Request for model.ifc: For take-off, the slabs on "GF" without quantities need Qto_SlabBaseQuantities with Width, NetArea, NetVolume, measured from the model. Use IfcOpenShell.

First a look at what the model holds.

```python
import ifcopenshell
import ifcopenshell.util.element
import ifcopenshell.util.unit

model = ifcopenshell.open("model.ifc")
print(model.schema)
for unit_type in ("LENGTHUNIT", "AREAUNIT", "VOLUMEUNIT"):
    print(unit_type, ifcopenshell.util.unit.calculate_unit_scale(model, unit_type))
storey = next(s for s in model.by_type("IfcBuildingStorey") if s.Name == "GF")
slabs = [e for e in ifcopenshell.util.element.get_decomposition(storey) if e.is_a("IfcSlab")]
for e in sorted(slabs, key=lambda e: e.id()):
    print(e.id(), e.is_a(), e.Name, list(ifcopenshell.util.element.get_psets(e, qtos_only=True)), sep=" | ")
```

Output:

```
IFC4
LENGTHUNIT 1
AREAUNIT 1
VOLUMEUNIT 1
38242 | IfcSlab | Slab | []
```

```python
import ifcopenshell
import ifcopenshell.api.pset
import ifcopenshell.geom
import ifcopenshell.util.element
import ifcopenshell.util.shape
import ifcopenshell.util.unit

model = ifcopenshell.open("model.ifc")
unit_scale = ifcopenshell.util.unit.calculate_unit_scale(model)
area_scale = ifcopenshell.util.unit.calculate_unit_scale(model, "AREAUNIT")
volume_scale = ifcopenshell.util.unit.calculate_unit_scale(model, "VOLUMEUNIT")
settings = ifcopenshell.geom.settings()

storey = next(s for s in model.by_type("IfcBuildingStorey") if s.Name == "GF")
slabs = [e for e in ifcopenshell.util.element.get_decomposition(storey) if e.is_a("IfcSlab")]

for e in sorted(slabs, key=lambda e: e.id()):
    if ifcopenshell.util.element.get_psets(e, qtos_only=True, should_inherit=False):
        continue
    # Geometry comes back in metres, in the element's own axes.
    shape = ifcopenshell.geom.create_shape(settings, e)
    values = {
        "Width": ifcopenshell.util.shape.get_z(shape.geometry) / unit_scale,
        "NetArea": ifcopenshell.util.shape.get_footprint_area(shape.geometry) / area_scale,
        "NetVolume": ifcopenshell.util.shape.get_volume(shape.geometry) / volume_scale,
    }
    qto = ifcopenshell.api.pset.add_qto(model, product=e, name="Qto_SlabBaseQuantities")
    ifcopenshell.api.pset.edit_qto(model, qto=qto, properties=values)
    print(e.id(), {k: round(v, 3) for k, v in values.items()})

model.write("model-out.ifc")
```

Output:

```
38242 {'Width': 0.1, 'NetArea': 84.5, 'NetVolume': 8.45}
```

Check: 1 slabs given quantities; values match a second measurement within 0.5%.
